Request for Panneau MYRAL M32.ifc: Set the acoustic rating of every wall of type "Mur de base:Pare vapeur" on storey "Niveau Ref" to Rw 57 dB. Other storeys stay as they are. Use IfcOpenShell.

First a look at what the model holds.

```python
import ifcopenshell
import ifcopenshell.util.element

model = ifcopenshell.open("Panneau MYRAL M32.ifc")
print(model.schema)
storey = next(s for s in model.by_type("IfcBuildingStorey") if s.Name == "Niveau Ref")
walls = [e for e in ifcopenshell.util.element.get_decomposition(storey) if e.is_a("IfcWall")]
seen = {}
for e in walls:
    element_type = ifcopenshell.util.element.get_type(e)
    key = (element_type.Name if element_type != e and element_type else None, ifcopenshell.util.element.get_pset(e, "Pset_WallCommon", "AcousticRating"))
    seen[key] = seen.get(key, 0) + 1
for (name, value), count in sorted(seen.items(), key=str):
    print(count, "x", name, "|", value)
```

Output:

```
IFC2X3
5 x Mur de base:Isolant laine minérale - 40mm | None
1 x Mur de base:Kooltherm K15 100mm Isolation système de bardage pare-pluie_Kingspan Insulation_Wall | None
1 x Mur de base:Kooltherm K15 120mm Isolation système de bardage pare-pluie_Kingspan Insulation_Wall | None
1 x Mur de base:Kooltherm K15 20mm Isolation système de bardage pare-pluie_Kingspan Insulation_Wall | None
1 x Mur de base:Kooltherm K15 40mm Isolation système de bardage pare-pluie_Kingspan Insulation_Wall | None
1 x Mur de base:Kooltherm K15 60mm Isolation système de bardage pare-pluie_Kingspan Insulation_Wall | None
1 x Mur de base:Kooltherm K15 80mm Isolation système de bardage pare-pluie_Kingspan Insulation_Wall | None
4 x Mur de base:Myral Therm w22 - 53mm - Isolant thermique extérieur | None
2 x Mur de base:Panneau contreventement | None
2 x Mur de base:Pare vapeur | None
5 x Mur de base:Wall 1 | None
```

```python
import ifcopenshell
import ifcopenshell.api.pset
import ifcopenshell.util.element

model = ifcopenshell.open("Panneau MYRAL M32.ifc")

storey = next(s for s in model.by_type("IfcBuildingStorey") if s.Name == "Niveau Ref")
walls = [e for e in ifcopenshell.util.element.get_decomposition(storey) if e.is_a("IfcWall")]

count = 0
for e in walls:
    element_type = ifcopenshell.util.element.get_type(e)
    if element_type in (None, e) or element_type.Name != "Mur de base:Pare vapeur":
        continue
    # add_pset returns the element's existing set when there is one.
    pset = ifcopenshell.api.pset.add_pset(model, product=e, name="Pset_WallCommon")
    ifcopenshell.api.pset.edit_pset(model, pset=pset, properties={"AcousticRating": "Rw 57 dB"})
    count += 1

print(count, "walls updated")

model.write("Panneau MYRAL M32_rev.ifc")
```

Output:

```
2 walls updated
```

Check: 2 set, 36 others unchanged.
